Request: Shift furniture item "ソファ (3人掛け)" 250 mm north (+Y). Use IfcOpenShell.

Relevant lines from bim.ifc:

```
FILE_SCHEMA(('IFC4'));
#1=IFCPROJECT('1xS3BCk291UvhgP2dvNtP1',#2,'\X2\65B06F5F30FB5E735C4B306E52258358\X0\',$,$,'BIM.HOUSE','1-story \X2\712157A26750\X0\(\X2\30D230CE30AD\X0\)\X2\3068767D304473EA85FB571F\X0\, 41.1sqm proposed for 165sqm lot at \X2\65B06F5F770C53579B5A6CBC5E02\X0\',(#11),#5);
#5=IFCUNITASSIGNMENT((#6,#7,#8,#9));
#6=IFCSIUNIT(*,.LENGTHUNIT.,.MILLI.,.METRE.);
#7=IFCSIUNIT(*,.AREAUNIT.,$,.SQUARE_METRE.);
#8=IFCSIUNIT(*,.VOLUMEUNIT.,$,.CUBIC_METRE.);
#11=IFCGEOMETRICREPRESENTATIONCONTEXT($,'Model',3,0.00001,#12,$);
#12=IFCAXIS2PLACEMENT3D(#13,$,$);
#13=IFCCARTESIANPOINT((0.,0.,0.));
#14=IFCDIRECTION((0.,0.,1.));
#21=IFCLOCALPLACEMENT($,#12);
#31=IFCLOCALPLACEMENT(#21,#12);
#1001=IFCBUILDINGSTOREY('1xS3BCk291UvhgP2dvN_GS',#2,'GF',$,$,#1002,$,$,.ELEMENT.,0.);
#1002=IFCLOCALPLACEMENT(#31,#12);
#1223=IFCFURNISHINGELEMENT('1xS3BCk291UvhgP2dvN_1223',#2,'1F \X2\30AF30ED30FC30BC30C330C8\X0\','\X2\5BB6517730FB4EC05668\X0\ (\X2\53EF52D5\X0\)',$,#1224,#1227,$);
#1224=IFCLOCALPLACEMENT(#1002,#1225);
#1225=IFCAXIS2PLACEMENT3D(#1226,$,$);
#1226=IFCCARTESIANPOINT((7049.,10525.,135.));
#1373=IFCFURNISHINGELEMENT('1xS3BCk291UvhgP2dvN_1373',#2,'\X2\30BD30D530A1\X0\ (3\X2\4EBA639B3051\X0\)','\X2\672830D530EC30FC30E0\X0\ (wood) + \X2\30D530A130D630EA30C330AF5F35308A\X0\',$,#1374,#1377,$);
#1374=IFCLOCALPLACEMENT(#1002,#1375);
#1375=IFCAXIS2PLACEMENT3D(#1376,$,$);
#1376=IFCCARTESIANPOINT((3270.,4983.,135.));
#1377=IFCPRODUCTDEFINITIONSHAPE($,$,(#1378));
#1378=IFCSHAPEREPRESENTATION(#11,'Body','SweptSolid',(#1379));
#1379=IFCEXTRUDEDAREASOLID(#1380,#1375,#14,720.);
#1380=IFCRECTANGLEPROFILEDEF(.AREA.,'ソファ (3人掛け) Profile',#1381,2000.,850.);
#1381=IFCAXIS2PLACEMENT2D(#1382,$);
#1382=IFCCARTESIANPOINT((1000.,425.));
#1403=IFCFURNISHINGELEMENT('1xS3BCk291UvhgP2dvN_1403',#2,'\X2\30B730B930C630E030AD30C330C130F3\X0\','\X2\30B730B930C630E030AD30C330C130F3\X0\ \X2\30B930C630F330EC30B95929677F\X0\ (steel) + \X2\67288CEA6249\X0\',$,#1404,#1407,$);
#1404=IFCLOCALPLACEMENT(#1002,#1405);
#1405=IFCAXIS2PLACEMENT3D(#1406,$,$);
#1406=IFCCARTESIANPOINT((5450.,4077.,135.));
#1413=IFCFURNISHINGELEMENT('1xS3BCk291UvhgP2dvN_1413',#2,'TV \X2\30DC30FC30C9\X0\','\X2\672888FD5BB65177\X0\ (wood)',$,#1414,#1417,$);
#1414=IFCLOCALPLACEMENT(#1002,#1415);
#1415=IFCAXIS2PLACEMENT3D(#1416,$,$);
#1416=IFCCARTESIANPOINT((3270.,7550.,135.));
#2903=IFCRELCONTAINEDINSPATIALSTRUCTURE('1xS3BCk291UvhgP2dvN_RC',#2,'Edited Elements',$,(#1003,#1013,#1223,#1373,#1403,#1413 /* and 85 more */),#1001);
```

```python
import ifcopenshell
import ifcopenshell.api.geometry
import ifcopenshell.util.placement

model = ifcopenshell.open("bim.ifc")

item = model.by_guid("1xS3BCk291UvhgP2dvN_1373")
matrix = ifcopenshell.util.placement.get_local_placement(item.ObjectPlacement)
matrix[1, 3] += 250.0
ifcopenshell.api.geometry.edit_object_placement(model, product=item, matrix=matrix, is_si=False)

print(ifcopenshell.util.placement.get_local_placement(item.ObjectPlacement).round(3) + 0.0)

model.write("bim_edited.ifc")
```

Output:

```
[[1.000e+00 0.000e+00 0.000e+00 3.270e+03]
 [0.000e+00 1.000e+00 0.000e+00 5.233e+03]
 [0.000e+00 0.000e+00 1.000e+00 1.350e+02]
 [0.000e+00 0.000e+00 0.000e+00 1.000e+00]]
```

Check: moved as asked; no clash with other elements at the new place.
